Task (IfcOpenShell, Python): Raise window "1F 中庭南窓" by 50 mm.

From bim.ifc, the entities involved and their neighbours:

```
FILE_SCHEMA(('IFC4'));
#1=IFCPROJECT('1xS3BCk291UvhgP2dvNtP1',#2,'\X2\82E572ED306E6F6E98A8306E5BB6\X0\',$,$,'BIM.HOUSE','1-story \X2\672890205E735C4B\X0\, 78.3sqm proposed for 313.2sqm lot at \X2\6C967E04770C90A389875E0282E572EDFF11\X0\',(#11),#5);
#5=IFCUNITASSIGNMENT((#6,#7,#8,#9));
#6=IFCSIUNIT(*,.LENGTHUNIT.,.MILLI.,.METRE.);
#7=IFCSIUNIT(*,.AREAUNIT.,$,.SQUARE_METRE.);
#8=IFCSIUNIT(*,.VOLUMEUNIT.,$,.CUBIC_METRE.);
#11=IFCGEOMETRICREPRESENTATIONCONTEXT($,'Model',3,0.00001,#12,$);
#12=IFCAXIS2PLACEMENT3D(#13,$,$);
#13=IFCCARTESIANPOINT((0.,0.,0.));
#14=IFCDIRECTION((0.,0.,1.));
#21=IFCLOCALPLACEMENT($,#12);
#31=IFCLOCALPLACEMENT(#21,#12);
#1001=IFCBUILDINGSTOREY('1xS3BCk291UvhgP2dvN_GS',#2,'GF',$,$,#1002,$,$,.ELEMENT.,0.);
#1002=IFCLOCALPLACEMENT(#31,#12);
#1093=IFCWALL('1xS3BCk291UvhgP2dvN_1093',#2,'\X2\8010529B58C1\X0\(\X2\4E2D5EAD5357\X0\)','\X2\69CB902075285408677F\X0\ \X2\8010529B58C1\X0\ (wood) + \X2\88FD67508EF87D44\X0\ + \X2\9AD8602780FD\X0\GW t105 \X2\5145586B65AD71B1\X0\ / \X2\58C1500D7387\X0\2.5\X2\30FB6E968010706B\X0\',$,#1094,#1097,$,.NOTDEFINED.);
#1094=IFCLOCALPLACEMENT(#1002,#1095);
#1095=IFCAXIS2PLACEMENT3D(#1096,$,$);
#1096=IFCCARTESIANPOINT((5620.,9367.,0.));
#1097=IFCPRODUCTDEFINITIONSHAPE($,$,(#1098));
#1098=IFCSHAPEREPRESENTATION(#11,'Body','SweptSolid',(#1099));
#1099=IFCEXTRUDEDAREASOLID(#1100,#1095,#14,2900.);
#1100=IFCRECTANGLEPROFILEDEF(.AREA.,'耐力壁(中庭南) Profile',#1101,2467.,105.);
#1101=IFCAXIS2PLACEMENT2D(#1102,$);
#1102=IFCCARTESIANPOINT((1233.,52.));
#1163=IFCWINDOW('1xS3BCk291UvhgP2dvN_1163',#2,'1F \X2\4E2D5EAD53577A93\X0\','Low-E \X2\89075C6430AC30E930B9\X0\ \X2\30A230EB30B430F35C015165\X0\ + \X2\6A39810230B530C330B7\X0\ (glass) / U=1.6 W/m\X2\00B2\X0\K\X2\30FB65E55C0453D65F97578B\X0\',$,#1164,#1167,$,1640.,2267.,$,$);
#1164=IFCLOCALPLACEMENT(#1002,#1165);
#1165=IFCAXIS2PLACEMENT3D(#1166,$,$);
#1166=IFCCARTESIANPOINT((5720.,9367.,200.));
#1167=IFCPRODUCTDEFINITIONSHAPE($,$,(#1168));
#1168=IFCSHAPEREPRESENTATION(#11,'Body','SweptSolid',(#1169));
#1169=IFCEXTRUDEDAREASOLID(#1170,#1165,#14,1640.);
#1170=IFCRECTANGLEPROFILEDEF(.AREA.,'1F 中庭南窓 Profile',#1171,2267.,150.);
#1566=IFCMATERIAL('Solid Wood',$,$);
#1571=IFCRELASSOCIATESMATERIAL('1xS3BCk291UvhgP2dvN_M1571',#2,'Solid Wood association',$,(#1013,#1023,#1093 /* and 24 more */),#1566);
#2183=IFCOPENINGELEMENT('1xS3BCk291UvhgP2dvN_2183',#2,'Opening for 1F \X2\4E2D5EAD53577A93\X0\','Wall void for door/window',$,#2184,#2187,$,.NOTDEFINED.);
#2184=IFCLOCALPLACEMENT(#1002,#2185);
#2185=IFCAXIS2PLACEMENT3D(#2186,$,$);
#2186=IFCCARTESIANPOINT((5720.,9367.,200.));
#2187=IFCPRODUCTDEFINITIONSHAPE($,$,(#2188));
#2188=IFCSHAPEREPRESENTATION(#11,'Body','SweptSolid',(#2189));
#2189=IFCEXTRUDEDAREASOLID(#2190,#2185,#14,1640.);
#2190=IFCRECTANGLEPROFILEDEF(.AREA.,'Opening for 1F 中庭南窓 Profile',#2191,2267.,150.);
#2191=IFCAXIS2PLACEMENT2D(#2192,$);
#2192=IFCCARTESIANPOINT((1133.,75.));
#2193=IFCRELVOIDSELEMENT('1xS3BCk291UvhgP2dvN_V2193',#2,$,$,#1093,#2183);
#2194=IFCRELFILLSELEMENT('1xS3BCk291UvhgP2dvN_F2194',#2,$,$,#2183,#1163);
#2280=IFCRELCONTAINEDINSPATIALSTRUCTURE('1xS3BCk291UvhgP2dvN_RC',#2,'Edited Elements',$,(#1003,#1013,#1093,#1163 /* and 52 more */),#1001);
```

```python
import numpy as np
import ifcopenshell
import ifcopenshell.api.geometry
import ifcopenshell.util.placement
import ifcopenshell.util.unit

model = ifcopenshell.open("bim.ifc")
unit_scale = ifcopenshell.util.unit.calculate_unit_scale(model)

window = model.by_guid("1xS3BCk291UvhgP2dvN_1163")
opening = window.FillsVoids[0].RelatingOpeningElement
dz = 50.0

shift = np.array([0.0, 0.0, dz])
# The window is not placed relative to its opening, so move both.
for product in (opening, window):
    matrix = ifcopenshell.util.placement.get_local_placement(product.ObjectPlacement)
    matrix[:3, 3] += shift
    ifcopenshell.api.geometry.edit_object_placement(model, product=product, matrix=matrix, is_si=False)

print(f"moved by {dz * unit_scale:+.3f} m")

model.write("bim_v2.ifc")
```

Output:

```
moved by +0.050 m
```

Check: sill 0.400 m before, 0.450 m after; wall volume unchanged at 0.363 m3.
